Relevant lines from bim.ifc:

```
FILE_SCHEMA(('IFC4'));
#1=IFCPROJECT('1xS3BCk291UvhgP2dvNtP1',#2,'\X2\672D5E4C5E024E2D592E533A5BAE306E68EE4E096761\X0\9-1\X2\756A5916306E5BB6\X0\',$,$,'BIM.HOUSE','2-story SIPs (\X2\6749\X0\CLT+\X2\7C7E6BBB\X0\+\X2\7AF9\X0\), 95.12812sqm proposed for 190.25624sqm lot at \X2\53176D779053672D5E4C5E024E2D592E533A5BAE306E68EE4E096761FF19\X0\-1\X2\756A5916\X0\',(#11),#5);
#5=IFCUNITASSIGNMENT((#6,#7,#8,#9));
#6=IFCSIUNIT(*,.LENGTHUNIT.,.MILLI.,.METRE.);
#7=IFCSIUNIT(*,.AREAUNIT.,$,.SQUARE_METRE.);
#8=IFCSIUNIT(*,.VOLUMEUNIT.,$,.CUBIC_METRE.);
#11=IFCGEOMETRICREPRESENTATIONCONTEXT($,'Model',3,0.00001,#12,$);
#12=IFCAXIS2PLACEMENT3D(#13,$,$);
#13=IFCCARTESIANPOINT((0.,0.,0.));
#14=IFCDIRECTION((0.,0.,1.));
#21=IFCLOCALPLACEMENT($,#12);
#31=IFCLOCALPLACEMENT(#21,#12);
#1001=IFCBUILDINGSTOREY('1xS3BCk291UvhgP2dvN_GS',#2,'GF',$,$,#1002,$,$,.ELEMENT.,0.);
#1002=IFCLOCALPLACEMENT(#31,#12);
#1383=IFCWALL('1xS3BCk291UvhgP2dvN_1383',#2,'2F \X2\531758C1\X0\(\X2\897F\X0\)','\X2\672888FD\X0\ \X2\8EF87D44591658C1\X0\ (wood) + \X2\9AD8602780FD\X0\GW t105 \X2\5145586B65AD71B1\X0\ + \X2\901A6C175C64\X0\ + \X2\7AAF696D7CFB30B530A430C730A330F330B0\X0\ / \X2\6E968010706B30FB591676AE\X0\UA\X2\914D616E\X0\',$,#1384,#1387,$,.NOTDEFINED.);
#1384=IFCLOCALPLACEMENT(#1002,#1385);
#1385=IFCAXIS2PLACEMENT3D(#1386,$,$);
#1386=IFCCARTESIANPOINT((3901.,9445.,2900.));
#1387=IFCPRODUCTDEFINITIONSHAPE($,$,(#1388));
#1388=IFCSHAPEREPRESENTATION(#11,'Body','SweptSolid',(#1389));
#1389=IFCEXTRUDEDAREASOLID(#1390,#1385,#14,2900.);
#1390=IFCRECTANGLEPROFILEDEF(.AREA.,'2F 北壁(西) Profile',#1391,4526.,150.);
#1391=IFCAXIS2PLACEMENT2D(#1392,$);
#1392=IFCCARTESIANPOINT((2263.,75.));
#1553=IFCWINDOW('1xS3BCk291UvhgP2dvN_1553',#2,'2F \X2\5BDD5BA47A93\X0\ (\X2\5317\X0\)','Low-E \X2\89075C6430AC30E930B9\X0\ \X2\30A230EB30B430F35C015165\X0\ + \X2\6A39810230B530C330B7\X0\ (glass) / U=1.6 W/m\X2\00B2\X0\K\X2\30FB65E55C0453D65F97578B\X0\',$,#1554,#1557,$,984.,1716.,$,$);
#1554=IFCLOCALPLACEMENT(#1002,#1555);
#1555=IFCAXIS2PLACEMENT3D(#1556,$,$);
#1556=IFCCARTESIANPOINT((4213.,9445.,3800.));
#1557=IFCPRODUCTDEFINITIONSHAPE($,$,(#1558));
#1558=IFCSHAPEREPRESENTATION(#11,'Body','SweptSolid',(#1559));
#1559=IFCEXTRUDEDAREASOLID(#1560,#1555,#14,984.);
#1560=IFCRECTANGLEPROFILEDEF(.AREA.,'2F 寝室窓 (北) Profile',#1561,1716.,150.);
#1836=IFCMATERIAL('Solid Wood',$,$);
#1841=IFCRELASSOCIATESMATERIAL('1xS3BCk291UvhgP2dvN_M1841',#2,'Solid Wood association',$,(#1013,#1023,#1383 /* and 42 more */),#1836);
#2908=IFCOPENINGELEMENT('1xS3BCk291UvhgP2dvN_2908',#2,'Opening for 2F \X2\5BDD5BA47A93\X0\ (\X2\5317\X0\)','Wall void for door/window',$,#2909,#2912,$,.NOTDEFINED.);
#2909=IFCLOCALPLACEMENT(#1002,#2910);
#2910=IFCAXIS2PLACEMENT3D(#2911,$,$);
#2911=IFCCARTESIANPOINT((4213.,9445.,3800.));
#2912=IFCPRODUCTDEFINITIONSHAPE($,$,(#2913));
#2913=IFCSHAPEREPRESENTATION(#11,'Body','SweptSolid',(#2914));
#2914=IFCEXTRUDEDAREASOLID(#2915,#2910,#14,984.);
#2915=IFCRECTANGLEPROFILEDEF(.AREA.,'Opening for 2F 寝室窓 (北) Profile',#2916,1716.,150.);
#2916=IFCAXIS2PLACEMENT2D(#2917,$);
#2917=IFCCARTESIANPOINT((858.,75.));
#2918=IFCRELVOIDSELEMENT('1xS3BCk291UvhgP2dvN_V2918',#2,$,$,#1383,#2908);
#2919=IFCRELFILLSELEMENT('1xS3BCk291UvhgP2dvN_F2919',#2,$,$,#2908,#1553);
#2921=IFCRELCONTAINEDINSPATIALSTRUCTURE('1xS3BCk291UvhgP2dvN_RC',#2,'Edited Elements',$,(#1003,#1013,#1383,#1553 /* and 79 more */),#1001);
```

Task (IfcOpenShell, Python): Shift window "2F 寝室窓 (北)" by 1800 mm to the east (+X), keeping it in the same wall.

```python
import ifcopenshell
import ifcopenshell.api.geometry
import ifcopenshell.util.placement

model = ifcopenshell.open("bim.ifc")

window = model.by_guid("1xS3BCk291UvhgP2dvN_1553")
opening = window.FillsVoids[0].RelatingOpeningElement
wall = opening.VoidsElements[0].RelatingBuildingElement

wall_matrix = ifcopenshell.util.placement.get_local_placement(wall.ObjectPlacement)
shift = wall_matrix[:3, 0] * 1800.0
before = ifcopenshell.util.placement.get_local_placement(window.ObjectPlacement)[:3, 3].copy()

# The window is not placed relative to its opening, so move both.
for product in (opening, window):
    matrix = ifcopenshell.util.placement.get_local_placement(product.ObjectPlacement)
    matrix[:3, 3] += shift
    ifcopenshell.api.geometry.edit_object_placement(model, product=product, matrix=matrix, is_si=False)

after = ifcopenshell.util.placement.get_local_placement(window.ObjectPlacement)[:3, 3]
print("window moved by", (after - before).round(3) + 0.0)

model.write("bim_edited.ifc")
```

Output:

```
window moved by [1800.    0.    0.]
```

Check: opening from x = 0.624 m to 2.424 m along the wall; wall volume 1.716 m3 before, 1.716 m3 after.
